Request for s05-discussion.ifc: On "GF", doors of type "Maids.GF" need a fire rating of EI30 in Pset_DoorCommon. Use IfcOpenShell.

First a look at what the model holds.

```python
import ifcopenshell
import ifcopenshell.util.element

model = ifcopenshell.open("s05-discussion.ifc")
print(model.schema)
storey = next(s for s in model.by_type("IfcBuildingStorey") if s.Name == "GF")
doors = [e for e in ifcopenshell.util.element.get_decomposition(storey) if e.is_a("IfcDoor")]
seen = {}
for e in doors:
    element_type = ifcopenshell.util.element.get_type(e)
    key = (element_type.Name if element_type != e and element_type else None, ifcopenshell.util.element.get_pset(e, "Pset_DoorCommon", "FireRating"))
    seen[key] = seen.get(key, 0) + 1
for (name, value), count in sorted(seen.items(), key=str):
    print(count, "x", name, "|", value)
```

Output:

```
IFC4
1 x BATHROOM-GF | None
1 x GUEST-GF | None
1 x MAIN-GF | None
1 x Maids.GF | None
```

```python
import ifcopenshell
import ifcopenshell.api.pset
import ifcopenshell.util.element

model = ifcopenshell.open("s05-discussion.ifc")

storey = next(s for s in model.by_type("IfcBuildingStorey") if s.Name == "GF")
doors = [e for e in ifcopenshell.util.element.get_decomposition(storey) if e.is_a("IfcDoor")]

count = 0
for e in doors:
    element_type = ifcopenshell.util.element.get_type(e)
    if element_type in (None, e) or element_type.Name != "Maids.GF":
        continue
    # add_pset returns the element's existing set when there is one.
    pset = ifcopenshell.api.pset.add_pset(model, product=e, name="Pset_DoorCommon")
    ifcopenshell.api.pset.edit_pset(model, pset=pset, properties={"FireRating": "EI30"})
    count += 1

print(count, "doors updated")

model.write("s05-discussion_updated.ifc")
```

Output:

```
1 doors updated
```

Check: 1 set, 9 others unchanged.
